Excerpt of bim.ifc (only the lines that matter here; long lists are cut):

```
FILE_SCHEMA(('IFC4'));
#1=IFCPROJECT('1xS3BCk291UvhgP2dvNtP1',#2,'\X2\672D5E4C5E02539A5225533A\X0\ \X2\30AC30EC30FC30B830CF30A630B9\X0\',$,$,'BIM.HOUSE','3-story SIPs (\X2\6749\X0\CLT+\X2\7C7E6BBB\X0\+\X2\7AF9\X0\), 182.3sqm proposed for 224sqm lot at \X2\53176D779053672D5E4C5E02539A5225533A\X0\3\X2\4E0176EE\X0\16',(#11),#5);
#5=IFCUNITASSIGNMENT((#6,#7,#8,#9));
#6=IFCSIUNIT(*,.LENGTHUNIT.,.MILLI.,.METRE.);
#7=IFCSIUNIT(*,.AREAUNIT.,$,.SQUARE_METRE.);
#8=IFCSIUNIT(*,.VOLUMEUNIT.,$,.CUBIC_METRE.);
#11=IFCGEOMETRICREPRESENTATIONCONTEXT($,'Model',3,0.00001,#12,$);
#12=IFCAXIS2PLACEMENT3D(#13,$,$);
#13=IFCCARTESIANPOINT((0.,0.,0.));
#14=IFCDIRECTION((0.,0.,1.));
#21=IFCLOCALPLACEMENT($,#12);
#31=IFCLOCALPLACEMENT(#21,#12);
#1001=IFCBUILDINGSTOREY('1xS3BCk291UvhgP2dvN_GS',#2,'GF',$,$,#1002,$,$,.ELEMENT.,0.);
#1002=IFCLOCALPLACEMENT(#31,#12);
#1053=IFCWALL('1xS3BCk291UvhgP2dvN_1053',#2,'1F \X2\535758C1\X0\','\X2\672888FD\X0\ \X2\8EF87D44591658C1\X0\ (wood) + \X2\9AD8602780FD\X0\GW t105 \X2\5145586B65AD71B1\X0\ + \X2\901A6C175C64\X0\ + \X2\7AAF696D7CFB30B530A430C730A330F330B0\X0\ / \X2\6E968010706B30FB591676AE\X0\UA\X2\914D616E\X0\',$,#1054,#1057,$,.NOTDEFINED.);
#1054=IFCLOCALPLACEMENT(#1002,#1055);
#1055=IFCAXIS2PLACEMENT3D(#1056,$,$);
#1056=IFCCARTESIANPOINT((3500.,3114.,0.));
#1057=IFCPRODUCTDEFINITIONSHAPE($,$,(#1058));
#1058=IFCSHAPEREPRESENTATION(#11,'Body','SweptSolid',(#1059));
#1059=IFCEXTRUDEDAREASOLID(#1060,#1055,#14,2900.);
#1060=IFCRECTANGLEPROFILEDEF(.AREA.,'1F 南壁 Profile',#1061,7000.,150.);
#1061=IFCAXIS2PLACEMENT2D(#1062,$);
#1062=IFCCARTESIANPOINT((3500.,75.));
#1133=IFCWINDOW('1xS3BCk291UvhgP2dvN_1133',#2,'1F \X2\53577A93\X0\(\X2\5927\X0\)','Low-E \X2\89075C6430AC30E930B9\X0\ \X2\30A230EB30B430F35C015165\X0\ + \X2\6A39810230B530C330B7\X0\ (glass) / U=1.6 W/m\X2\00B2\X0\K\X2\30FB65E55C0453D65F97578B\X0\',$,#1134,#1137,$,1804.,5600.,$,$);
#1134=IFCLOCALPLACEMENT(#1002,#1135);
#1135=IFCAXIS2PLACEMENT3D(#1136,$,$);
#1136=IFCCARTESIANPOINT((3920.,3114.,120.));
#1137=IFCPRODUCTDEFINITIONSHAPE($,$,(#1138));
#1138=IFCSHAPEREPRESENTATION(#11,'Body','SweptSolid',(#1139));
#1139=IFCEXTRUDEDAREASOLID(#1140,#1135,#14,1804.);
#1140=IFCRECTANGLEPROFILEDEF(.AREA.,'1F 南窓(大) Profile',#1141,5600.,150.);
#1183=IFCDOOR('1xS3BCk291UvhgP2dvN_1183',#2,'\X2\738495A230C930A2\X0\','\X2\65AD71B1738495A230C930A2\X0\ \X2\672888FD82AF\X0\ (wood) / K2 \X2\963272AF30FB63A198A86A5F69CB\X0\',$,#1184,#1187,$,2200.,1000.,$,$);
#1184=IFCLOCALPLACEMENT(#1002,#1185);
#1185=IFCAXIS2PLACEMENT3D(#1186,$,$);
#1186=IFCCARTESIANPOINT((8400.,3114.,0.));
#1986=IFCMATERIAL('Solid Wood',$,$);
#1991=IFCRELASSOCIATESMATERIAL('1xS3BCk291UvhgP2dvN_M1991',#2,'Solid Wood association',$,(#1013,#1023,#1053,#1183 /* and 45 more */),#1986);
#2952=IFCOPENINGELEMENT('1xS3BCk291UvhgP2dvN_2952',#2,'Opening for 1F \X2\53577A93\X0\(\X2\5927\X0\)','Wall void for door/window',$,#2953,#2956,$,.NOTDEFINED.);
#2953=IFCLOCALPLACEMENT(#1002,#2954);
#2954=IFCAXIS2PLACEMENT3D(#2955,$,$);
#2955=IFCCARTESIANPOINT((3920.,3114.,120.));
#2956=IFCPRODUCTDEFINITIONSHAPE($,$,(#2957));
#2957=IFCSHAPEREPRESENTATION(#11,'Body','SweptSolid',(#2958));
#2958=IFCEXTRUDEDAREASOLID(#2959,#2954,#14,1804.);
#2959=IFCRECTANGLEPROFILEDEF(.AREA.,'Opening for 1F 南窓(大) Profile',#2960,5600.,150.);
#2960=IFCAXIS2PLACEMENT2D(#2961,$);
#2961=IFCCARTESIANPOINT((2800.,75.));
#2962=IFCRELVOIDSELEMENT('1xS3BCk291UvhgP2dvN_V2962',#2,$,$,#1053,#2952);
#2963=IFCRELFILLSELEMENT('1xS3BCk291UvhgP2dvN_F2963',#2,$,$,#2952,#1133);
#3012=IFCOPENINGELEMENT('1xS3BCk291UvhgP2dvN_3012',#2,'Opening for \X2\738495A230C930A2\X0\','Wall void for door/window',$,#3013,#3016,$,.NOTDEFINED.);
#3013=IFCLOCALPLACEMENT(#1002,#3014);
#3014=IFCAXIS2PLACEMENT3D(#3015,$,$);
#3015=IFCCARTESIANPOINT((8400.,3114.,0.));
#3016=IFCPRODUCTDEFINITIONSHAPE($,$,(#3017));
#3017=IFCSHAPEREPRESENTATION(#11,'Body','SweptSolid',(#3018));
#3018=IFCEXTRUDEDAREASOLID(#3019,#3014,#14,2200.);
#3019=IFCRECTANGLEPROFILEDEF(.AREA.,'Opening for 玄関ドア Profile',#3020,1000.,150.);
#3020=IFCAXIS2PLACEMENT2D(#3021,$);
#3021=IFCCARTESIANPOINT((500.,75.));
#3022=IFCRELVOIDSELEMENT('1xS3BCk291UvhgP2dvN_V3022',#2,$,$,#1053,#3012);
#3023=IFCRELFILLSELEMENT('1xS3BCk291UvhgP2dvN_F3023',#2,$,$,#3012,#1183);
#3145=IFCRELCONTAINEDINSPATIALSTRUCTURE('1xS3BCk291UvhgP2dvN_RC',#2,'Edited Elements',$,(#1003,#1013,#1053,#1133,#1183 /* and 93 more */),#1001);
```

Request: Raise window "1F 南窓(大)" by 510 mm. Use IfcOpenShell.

```python
import numpy as np
import ifcopenshell
import ifcopenshell.api.geometry
import ifcopenshell.util.placement
import ifcopenshell.util.unit

model = ifcopenshell.open("bim.ifc")
unit_scale = ifcopenshell.util.unit.calculate_unit_scale(model)

window = model.by_guid("1xS3BCk291UvhgP2dvN_1133")
opening = window.FillsVoids[0].RelatingOpeningElement
dz = 0.51 / unit_scale

shift = np.array([0.0, 0.0, dz])
# The window is not placed relative to its opening, so move both.
for product in (opening, window):
    matrix = ifcopenshell.util.placement.get_local_placement(product.ObjectPlacement)
    matrix[:3, 3] += shift
    ifcopenshell.api.geometry.edit_object_placement(model, product=product, matrix=matrix, is_si=False)

print(f"moved by {dz * unit_scale:+.3f} m")

model.write("bim_rev.ifc")
```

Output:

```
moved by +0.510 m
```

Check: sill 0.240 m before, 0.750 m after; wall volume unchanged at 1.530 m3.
